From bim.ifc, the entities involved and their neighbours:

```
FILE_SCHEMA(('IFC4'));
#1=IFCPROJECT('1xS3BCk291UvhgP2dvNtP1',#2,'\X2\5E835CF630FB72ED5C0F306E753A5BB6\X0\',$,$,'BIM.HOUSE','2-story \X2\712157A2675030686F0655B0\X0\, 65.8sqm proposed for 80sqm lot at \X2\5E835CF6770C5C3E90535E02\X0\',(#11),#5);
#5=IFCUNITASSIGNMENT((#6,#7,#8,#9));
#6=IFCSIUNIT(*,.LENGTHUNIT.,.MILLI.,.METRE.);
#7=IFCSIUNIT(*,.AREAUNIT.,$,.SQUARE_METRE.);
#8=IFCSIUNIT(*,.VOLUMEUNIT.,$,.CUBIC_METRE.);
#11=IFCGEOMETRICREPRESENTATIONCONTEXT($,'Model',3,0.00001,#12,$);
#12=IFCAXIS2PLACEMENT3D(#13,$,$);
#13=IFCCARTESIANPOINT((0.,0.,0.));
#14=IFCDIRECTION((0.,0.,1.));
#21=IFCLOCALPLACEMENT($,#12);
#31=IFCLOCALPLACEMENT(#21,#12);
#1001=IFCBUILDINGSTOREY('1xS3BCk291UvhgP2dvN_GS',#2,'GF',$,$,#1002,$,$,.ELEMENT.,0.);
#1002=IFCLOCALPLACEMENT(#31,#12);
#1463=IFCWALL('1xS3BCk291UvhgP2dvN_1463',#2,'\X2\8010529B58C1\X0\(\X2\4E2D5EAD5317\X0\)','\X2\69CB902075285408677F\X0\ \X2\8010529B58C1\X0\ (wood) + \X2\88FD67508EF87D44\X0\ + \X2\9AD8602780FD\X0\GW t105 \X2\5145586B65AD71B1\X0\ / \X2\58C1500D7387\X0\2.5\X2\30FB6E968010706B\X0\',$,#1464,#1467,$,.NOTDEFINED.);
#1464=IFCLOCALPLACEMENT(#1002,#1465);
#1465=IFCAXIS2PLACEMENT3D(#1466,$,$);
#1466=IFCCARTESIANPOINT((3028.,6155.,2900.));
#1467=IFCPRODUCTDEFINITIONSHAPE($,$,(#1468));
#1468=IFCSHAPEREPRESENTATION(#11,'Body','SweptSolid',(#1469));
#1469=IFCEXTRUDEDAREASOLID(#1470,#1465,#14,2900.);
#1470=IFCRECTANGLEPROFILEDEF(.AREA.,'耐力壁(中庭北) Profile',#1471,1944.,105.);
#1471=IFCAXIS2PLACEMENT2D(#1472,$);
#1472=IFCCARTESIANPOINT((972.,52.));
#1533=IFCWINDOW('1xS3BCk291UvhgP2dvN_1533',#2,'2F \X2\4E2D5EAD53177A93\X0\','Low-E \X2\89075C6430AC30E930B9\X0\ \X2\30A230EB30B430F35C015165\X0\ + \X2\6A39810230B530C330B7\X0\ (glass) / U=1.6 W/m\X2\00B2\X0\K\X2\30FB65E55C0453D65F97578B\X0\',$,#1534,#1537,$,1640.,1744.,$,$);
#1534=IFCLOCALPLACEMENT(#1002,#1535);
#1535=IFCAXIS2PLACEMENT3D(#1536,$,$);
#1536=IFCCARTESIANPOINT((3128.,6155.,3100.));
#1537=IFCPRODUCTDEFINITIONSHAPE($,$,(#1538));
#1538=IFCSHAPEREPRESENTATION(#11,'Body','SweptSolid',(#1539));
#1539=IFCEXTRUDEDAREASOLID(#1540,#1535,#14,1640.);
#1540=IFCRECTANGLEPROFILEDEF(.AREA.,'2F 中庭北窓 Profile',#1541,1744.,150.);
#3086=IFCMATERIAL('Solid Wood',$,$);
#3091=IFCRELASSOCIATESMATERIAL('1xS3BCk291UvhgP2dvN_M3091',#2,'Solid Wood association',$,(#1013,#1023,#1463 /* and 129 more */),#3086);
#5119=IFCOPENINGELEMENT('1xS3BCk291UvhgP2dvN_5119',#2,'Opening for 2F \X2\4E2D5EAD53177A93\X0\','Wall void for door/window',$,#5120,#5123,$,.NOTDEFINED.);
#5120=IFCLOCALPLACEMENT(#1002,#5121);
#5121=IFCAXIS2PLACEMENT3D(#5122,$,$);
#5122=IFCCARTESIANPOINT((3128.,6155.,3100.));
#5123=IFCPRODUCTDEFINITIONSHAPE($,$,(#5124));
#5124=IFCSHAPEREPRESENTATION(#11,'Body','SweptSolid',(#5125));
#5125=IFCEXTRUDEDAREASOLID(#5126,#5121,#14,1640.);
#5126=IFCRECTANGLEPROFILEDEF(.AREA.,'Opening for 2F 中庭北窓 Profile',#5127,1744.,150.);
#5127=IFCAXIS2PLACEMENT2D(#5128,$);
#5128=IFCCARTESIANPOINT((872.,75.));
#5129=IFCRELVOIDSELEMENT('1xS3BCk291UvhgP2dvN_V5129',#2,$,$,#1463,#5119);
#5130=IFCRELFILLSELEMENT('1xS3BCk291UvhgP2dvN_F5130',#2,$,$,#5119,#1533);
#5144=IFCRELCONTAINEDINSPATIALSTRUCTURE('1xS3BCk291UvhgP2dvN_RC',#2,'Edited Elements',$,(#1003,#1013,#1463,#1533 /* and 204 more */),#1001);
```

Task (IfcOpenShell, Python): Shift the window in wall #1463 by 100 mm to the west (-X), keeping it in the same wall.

```python
import ifcopenshell
import ifcopenshell.api.geometry
import ifcopenshell.util.placement
import ifcopenshell.util.unit

model = ifcopenshell.open("bim.ifc")
unit_scale = ifcopenshell.util.unit.calculate_unit_scale(model)

window = model.by_guid("1xS3BCk291UvhgP2dvN_1533")
opening = window.FillsVoids[0].RelatingOpeningElement
wall = opening.VoidsElements[0].RelatingBuildingElement

wall_matrix = ifcopenshell.util.placement.get_local_placement(wall.ObjectPlacement)
shift = wall_matrix[:3, 0] * -0.1 / unit_scale
before = ifcopenshell.util.placement.get_local_placement(window.ObjectPlacement)[:3, 3].copy()

# The window is not placed relative to its opening, so move both.
for product in (opening, window):
    matrix = ifcopenshell.util.placement.get_local_placement(product.ObjectPlacement)
    matrix[:3, 3] += shift
    ifcopenshell.api.geometry.edit_object_placement(model, product=product, matrix=matrix, is_si=False)

after = ifcopenshell.util.placement.get_local_placement(window.ObjectPlacement)[:3, 3]
print("window moved by", (after - before).round(3) + 0.0)

model.write("bim-out.ifc")
```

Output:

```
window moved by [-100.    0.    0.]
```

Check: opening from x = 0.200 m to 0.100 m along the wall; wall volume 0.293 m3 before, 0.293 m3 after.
